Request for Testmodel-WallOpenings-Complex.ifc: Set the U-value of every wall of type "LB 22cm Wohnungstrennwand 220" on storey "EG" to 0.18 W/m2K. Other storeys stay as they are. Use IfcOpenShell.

First a look at what the model holds.

```python
import ifcopenshell
import ifcopenshell.util.element

model = ifcopenshell.open("Testmodel-WallOpenings-Complex.ifc")
print(model.schema)
storey = next(s for s in model.by_type("IfcBuildingStorey") if s.Name == "EG")
walls = [e for e in ifcopenshell.util.element.get_decomposition(storey) if e.is_a("IfcWall")]
seen = {}
for e in walls:
    element_type = ifcopenshell.util.element.get_type(e)
    key = (element_type.Name if element_type != e and element_type else None, ifcopenshell.util.element.get_pset(e, "Pset_WallCommon", "ThermalTransmittance"))
    seen[key] = seen.get(key, 0) + 1
for (name, value), count in sorted(seen.items(), key=str):
    print(count, "x", name, "|", value)
```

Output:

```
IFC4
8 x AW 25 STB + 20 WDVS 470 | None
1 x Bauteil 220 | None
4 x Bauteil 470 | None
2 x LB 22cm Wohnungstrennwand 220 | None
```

```python
import ifcopenshell
import ifcopenshell.api.pset
import ifcopenshell.util.element

model = ifcopenshell.open("Testmodel-WallOpenings-Complex.ifc")

storey = next(s for s in model.by_type("IfcBuildingStorey") if s.Name == "EG")
walls = [e for e in ifcopenshell.util.element.get_decomposition(storey) if e.is_a("IfcWall")]

count = 0
for e in walls:
    element_type = ifcopenshell.util.element.get_type(e)
    if element_type in (None, e) or element_type.Name != "LB 22cm Wohnungstrennwand 220":
        continue
    # add_pset returns the element's existing set when there is one.
    pset = ifcopenshell.api.pset.add_pset(model, product=e, name="Pset_WallCommon")
    ifcopenshell.api.pset.edit_pset(model, pset=pset, properties={"ThermalTransmittance": 0.18})
    count += 1

print(count, "walls updated")

model.write("Testmodel-WallOpenings-Complex-out.ifc")
```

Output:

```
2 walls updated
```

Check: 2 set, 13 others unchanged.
